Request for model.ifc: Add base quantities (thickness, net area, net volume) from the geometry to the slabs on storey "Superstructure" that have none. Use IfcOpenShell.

First a look at what the model holds.

```python
import ifcopenshell
import ifcopenshell.util.element
import ifcopenshell.util.unit

model = ifcopenshell.open("model.ifc")
print(model.schema)
for unit_type in ("LENGTHUNIT", "AREAUNIT", "VOLUMEUNIT"):
    print(unit_type, ifcopenshell.util.unit.calculate_unit_scale(model, unit_type))
storey = next(s for s in model.by_type("IfcBuildingStorey") if s.Name == "Superstructure")
slabs = [e for e in ifcopenshell.util.element.get_decomposition(storey) if e.is_a("IfcSlab")]
for e in sorted(slabs, key=lambda e: e.id()):
    print(e.id(), e.is_a(), e.Name, list(ifcopenshell.util.element.get_psets(e, qtos_only=True)), sep=" | ")
```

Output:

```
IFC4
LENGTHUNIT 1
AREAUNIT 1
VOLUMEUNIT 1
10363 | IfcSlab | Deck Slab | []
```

```python
import ifcopenshell
import ifcopenshell.api.pset
import ifcopenshell.geom
import ifcopenshell.util.element
import ifcopenshell.util.shape
import ifcopenshell.util.unit

model = ifcopenshell.open("model.ifc")
unit_scale = ifcopenshell.util.unit.calculate_unit_scale(model)
area_scale = ifcopenshell.util.unit.calculate_unit_scale(model, "AREAUNIT")
volume_scale = ifcopenshell.util.unit.calculate_unit_scale(model, "VOLUMEUNIT")
settings = ifcopenshell.geom.settings()

storey = next(s for s in model.by_type("IfcBuildingStorey") if s.Name == "Superstructure")
slabs = [e for e in ifcopenshell.util.element.get_decomposition(storey) if e.is_a("IfcSlab")]

for e in sorted(slabs, key=lambda e: e.id()):
    if ifcopenshell.util.element.get_psets(e, qtos_only=True, should_inherit=False):
        continue
    # Geometry comes back in metres, in the element's own axes.
    shape = ifcopenshell.geom.create_shape(settings, e)
    values = {
        "Width": ifcopenshell.util.shape.get_z(shape.geometry) / unit_scale,
        "NetArea": ifcopenshell.util.shape.get_footprint_area(shape.geometry) / area_scale,
        "NetVolume": ifcopenshell.util.shape.get_volume(shape.geometry) / volume_scale,
    }
    qto = ifcopenshell.api.pset.add_qto(model, product=e, name="Qto_SlabBaseQuantities")
    ifcopenshell.api.pset.edit_qto(model, qto=qto, properties=values)
    print(e.id(), {k: round(v, 3) for k, v in values.items()})

model.write("model_rev.ifc")
```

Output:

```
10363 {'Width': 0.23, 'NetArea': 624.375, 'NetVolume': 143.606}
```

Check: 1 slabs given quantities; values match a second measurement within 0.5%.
